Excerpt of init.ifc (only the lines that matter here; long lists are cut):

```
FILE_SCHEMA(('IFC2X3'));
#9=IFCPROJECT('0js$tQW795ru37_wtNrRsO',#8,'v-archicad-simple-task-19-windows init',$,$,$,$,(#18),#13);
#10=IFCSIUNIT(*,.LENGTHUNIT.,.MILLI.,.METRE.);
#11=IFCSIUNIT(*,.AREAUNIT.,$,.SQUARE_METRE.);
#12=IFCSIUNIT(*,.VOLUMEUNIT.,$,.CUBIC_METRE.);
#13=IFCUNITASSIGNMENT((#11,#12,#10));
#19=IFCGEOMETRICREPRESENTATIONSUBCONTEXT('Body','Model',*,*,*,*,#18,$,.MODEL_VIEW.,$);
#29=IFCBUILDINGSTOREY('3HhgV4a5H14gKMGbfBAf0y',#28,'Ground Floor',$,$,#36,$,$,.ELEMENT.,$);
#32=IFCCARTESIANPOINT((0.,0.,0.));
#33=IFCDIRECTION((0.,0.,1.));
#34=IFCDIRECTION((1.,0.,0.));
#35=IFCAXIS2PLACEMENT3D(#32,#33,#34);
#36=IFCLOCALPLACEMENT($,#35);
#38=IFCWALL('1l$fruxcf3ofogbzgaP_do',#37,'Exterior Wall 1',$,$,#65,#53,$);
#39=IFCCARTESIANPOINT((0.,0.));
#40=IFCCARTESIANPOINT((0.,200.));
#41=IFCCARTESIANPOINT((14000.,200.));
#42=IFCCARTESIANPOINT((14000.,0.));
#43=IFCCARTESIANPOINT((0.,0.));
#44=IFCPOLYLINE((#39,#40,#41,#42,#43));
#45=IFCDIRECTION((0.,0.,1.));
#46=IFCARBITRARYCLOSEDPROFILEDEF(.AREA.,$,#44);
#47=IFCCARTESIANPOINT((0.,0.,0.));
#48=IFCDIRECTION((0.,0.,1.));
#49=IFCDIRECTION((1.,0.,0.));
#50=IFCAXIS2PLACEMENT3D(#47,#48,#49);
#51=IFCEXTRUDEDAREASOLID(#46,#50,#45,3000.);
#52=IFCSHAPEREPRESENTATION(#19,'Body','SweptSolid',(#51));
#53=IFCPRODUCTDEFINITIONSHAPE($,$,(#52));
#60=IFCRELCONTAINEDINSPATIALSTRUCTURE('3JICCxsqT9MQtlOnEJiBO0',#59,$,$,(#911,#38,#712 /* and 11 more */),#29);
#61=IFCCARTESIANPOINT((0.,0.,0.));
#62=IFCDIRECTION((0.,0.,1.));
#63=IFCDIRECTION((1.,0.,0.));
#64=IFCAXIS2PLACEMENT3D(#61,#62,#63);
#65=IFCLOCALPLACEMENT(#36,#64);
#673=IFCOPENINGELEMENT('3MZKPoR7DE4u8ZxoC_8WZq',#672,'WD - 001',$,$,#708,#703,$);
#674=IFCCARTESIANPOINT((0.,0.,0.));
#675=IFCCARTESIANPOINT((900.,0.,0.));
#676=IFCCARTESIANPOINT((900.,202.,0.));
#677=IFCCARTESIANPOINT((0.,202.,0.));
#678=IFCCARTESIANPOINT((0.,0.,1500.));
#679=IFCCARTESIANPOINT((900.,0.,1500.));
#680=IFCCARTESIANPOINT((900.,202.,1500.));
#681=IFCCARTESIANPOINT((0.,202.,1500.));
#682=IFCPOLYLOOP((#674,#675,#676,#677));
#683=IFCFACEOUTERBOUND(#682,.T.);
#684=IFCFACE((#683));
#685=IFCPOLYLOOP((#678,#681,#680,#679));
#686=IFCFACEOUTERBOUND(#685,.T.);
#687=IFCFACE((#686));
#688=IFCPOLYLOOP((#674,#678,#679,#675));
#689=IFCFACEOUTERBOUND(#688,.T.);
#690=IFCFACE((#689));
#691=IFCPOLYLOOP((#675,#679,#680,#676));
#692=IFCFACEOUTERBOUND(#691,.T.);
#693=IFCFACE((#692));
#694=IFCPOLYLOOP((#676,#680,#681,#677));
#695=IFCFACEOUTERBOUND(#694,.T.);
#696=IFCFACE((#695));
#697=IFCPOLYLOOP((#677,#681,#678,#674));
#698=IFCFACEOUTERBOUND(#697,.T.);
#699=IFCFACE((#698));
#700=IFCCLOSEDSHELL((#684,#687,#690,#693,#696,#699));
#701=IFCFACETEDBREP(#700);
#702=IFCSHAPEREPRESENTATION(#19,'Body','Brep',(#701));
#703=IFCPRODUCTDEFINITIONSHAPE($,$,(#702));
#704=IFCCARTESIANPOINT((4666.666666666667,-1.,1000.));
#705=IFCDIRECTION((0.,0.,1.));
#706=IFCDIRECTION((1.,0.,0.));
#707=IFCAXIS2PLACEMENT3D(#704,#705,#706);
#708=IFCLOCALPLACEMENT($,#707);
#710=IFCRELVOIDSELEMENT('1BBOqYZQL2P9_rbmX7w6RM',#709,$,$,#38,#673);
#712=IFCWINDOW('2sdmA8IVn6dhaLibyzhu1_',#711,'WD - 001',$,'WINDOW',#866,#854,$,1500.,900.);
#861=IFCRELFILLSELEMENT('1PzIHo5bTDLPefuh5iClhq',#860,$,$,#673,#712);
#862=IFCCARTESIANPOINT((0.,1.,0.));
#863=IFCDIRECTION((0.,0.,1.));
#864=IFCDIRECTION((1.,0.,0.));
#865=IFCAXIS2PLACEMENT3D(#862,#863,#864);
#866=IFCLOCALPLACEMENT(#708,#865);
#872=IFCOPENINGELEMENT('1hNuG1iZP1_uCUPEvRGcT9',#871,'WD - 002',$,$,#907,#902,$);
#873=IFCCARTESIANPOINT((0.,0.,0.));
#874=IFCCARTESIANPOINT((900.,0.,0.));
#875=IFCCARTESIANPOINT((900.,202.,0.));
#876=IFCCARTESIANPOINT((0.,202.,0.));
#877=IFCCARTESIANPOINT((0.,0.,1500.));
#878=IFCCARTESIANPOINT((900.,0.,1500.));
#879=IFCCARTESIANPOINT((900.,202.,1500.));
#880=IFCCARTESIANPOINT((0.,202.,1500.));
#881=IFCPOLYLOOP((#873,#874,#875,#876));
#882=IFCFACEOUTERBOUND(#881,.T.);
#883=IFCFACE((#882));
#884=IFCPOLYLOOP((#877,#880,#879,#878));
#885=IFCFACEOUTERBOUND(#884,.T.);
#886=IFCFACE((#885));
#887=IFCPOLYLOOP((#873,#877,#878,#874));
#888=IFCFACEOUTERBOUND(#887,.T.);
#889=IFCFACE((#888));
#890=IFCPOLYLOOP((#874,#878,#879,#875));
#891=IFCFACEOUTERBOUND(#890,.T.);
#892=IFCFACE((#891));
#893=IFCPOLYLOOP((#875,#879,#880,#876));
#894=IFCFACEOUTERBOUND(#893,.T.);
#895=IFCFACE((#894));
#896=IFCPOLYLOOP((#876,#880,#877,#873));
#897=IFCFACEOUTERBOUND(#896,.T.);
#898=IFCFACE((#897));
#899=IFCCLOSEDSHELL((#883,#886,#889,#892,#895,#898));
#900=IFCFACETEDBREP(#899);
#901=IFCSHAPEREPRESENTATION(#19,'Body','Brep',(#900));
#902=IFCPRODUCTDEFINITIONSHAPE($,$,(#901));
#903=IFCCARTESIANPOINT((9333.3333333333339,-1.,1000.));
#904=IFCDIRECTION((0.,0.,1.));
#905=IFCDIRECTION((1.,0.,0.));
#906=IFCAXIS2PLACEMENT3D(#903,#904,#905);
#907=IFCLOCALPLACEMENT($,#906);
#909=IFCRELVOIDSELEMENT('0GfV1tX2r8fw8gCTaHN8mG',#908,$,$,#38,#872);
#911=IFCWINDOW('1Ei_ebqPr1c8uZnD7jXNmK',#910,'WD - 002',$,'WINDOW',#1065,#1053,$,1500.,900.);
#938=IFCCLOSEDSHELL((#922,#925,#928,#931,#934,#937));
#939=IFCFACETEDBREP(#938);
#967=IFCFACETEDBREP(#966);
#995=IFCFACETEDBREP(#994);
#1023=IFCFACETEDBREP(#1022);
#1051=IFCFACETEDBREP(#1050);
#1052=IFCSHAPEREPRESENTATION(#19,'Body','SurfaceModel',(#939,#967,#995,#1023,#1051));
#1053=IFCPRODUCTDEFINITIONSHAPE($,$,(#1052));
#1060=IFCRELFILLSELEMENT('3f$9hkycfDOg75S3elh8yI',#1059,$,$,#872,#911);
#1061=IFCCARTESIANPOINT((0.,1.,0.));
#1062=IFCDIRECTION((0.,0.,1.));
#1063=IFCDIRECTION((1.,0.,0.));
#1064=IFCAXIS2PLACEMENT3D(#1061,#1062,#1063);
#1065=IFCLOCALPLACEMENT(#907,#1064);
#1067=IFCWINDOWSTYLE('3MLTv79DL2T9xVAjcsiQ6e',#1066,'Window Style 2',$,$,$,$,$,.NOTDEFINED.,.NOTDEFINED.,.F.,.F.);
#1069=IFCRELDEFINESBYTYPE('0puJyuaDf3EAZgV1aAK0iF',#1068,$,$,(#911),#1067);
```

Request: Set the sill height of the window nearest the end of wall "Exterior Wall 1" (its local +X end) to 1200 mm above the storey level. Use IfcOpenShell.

```python
import numpy as np
import ifcopenshell
import ifcopenshell.api.geometry
import ifcopenshell.geom
import ifcopenshell.util.element
import ifcopenshell.util.placement
import ifcopenshell.util.shape
import ifcopenshell.util.unit

model = ifcopenshell.open("init.ifc")
unit_scale = ifcopenshell.util.unit.calculate_unit_scale(model)

window = model.by_id(911)
opening = window.FillsVoids[0].RelatingOpeningElement
storey = ifcopenshell.util.element.get_container(window, ifc_class="IfcBuildingStorey")
level = ifcopenshell.util.placement.get_local_placement(storey.ObjectPlacement)[2, 3]

# The opening's origin need not be at the sill, so measure its lowest point.
shape = ifcopenshell.geom.create_shape(ifcopenshell.geom.settings(), opening)
bottom = ifcopenshell.util.shape.get_shape_bottom_elevation(shape, shape.geometry) / unit_scale
dz = level + 1.2 / unit_scale - bottom

shift = np.array([0.0, 0.0, dz])
# The window is placed relative to its opening, so it follows when the opening moves.
matrix = ifcopenshell.util.placement.get_local_placement(opening.ObjectPlacement)
matrix[:3, 3] += shift
ifcopenshell.api.geometry.edit_object_placement(
    model, product=opening, matrix=matrix, is_si=False, should_transform_children=True
)

print(f"moved by {dz * unit_scale:+.3f} m")

model.write("init_rev.ifc")
```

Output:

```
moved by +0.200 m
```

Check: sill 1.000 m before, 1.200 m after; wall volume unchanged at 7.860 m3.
